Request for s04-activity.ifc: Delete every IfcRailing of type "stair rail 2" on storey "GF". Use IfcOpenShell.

First a look at what the model holds.

```python
import ifcopenshell
import ifcopenshell.util.element

model = ifcopenshell.open("s04-activity.ifc")
print(model.schema)
storey = next(s for s in model.by_type("IfcBuildingStorey") if s.Name == "GF")
railings = [e for e in ifcopenshell.util.element.get_decomposition(storey) if e.is_a("IfcRailing")]
seen = {}
for e in railings:
    element_type = ifcopenshell.util.element.get_type(e)
    name = element_type.Name if element_type not in (None, e) else None
    seen[name] = seen.get(name, 0) + 1
for name, count in sorted(seen.items(), key=str):
    print(count, "x", name)
```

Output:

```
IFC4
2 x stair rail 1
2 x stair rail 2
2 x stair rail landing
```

```python
import ifcopenshell
import ifcopenshell.api.root
import ifcopenshell.util.element

model = ifcopenshell.open("s04-activity.ifc")

storey = next(s for s in model.by_type("IfcBuildingStorey") if s.Name == "GF")
railings = [e for e in ifcopenshell.util.element.get_decomposition(storey) if e.is_a("IfcRailing")]
targets = [e for e in railings if (t := ifcopenshell.util.element.get_type(e)) not in (None, e) and t.Name == "stair rail 2"]

for e in targets:
    ifcopenshell.api.root.remove_product(model, product=e)
print(len(targets), "removed")

model.write("s04-activity_v2.ifc")
```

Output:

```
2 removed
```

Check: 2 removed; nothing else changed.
